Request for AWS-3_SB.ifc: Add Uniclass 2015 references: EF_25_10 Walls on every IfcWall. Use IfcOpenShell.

First a look at what the model holds.

```python
import ifcopenshell

model = ifcopenshell.open("AWS-3_SB.ifc")
print(model.schema)
print("classifications:", [c.Name for c in model.by_type("IfcClassification")])
for ifc_class in ("IfcDoor", "IfcRoof", "IfcStair", "IfcWall", "IfcWindow"):
    print(ifc_class, len(model.by_type(ifc_class)))
```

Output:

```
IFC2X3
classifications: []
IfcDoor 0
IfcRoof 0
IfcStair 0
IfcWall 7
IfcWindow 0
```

```python
import ifcopenshell
import ifcopenshell.api.classification

model = ifcopenshell.open("AWS-3_SB.ifc")

# IFC2X3 requires Source and Edition and has no link from the project to the system.
system = model.create_entity("IfcClassification", Source="NBS", Edition="2015", Name="Uniclass 2015")

codes = {
    "IfcWall": ("EF_25_10", "Walls"),
}
for ifc_class, (code, name) in codes.items():
    products = model.by_type(ifc_class)
    ifcopenshell.api.classification.add_reference(
        model, products=products, classification=system, identification=code, name=name
    )
    print(code, len(products))

model.write("AWS-3_SB_updated.ifc")
```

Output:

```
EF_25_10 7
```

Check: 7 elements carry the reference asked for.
